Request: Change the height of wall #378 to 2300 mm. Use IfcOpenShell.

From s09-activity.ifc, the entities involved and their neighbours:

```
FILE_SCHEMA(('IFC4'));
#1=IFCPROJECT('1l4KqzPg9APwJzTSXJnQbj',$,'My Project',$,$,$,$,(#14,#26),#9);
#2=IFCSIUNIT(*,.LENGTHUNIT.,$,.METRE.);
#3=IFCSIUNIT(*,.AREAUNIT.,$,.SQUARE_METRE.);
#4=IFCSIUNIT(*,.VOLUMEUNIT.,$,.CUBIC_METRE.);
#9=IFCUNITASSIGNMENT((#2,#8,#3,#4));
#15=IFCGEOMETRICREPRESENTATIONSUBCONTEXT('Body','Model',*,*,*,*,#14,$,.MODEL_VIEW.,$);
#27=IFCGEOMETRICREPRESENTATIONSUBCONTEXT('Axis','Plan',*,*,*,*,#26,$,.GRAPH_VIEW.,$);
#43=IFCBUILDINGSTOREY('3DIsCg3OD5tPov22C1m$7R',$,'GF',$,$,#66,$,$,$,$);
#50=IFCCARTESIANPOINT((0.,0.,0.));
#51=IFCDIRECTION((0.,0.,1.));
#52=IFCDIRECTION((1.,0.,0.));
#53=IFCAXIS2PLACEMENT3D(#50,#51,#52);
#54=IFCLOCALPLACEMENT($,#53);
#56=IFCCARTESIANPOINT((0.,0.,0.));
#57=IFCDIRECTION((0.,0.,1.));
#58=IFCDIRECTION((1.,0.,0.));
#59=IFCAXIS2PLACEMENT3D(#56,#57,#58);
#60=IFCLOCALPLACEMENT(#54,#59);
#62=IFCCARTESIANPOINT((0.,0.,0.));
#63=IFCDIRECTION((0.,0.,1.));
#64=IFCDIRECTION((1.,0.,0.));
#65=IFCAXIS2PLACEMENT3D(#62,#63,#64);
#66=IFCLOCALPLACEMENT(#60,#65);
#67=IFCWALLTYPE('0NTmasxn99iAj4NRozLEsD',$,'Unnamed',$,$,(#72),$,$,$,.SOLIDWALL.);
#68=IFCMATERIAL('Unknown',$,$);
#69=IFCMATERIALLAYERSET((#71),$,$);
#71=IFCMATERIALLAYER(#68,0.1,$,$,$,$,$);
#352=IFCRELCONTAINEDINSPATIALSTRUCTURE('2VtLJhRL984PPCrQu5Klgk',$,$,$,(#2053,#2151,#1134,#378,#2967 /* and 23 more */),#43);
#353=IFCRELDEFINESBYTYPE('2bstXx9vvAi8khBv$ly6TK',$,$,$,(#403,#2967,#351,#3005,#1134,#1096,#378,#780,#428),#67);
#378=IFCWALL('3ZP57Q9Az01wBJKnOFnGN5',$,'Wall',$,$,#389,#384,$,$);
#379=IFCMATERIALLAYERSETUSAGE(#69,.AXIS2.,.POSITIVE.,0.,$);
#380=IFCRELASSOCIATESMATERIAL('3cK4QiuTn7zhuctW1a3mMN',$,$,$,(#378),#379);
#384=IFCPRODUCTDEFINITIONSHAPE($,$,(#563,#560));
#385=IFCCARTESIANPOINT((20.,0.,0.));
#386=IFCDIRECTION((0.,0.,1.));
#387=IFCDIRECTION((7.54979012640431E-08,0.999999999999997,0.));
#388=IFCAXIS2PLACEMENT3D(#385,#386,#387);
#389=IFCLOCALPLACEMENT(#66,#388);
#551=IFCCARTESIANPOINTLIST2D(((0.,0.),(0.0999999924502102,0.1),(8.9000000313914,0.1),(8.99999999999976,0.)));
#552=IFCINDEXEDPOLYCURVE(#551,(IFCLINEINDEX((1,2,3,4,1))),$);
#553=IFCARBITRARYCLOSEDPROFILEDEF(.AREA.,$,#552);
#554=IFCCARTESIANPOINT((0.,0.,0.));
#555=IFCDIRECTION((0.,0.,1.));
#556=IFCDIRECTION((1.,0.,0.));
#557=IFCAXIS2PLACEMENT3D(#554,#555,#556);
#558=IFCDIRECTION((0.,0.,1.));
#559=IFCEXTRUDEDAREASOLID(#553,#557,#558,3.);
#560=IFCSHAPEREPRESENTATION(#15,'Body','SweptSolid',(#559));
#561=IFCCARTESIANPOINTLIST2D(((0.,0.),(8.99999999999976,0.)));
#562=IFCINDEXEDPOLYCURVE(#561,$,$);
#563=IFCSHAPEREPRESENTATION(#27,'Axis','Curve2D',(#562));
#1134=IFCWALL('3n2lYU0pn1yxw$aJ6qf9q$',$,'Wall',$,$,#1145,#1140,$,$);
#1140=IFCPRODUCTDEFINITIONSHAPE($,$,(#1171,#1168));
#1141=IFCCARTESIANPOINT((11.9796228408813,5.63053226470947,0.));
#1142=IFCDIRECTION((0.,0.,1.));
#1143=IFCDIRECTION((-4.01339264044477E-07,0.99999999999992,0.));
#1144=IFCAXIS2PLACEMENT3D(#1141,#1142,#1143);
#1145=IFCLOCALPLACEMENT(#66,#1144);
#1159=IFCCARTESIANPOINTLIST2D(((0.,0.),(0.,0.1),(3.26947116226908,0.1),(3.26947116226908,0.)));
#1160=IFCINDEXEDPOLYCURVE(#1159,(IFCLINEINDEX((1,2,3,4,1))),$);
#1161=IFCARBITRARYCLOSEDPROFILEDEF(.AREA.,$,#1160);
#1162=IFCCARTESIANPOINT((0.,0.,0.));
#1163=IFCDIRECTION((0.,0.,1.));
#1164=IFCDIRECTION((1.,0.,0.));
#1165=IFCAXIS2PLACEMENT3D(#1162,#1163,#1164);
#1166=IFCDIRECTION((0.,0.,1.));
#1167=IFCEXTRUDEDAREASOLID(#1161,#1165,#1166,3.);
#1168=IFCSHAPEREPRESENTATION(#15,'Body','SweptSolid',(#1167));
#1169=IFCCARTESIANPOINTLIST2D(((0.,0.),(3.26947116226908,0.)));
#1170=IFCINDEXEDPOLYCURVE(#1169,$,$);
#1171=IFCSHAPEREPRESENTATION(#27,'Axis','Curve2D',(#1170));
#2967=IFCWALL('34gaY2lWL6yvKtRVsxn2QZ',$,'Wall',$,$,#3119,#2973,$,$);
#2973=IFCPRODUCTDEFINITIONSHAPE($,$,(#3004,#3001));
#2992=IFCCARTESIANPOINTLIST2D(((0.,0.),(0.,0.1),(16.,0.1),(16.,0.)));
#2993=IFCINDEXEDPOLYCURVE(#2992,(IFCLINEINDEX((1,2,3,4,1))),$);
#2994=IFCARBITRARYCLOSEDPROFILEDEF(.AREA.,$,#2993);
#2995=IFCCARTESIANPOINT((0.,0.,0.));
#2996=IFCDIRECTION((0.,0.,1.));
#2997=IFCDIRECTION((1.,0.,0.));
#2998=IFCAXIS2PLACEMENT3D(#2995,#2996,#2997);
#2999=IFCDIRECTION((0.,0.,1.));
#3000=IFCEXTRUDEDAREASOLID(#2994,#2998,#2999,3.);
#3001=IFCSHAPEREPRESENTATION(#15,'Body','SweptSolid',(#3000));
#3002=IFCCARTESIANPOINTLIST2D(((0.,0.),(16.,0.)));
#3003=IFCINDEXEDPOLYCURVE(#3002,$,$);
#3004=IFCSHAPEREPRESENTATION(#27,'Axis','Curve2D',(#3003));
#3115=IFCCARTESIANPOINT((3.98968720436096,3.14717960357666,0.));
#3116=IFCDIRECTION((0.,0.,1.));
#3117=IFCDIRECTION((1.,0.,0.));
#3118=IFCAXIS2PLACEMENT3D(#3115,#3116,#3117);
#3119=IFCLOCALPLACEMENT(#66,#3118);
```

```python
import ifcopenshell
import ifcopenshell.geom
import ifcopenshell.util.representation
import ifcopenshell.util.shape
import ifcopenshell.util.unit

model = ifcopenshell.open("s09-activity.ifc")
unit_scale = ifcopenshell.util.unit.calculate_unit_scale(model)
settings = ifcopenshell.geom.settings()


def volume(element):
    """Net volume in cubic metres, openings subtracted."""
    shape = ifcopenshell.geom.create_shape(settings, element)
    return ifcopenshell.util.shape.get_volume(shape.geometry)


wall = model.by_id(378)
before = volume(wall)

body = ifcopenshell.util.representation.get_representation(wall, "Model", "Body")
solid = body.Items[0]
old_height = solid.Depth
solid.Depth = 2.3 / unit_scale
after = volume(wall)

print(f"height {old_height:g} -> {solid.Depth:g}, volume {before:.3f} -> {after:.3f} m3")

model.write("s09-activity_edited.ifc")
```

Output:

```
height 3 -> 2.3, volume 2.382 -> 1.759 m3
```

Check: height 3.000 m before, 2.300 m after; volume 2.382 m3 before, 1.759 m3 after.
